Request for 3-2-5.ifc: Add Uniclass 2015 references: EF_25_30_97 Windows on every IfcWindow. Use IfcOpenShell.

First a look at what the model holds.

```python
import ifcopenshell

model = ifcopenshell.open("3-2-5.ifc")
print(model.schema)
print("classifications:", [c.Name for c in model.by_type("IfcClassification")])
for ifc_class in ("IfcDoor", "IfcRoof", "IfcStair", "IfcWall", "IfcWindow"):
    print(ifc_class, len(model.by_type(ifc_class)))
```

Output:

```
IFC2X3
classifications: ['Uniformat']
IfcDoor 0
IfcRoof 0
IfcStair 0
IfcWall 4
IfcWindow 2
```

```python
import ifcopenshell
import ifcopenshell.api.classification

model = ifcopenshell.open("3-2-5.ifc")

# IFC2X3 requires Source and Edition and has no link from the project to the system.
system = model.create_entity("IfcClassification", Source="NBS", Edition="2015", Name="Uniclass 2015")

codes = {
    "IfcWindow": ("EF_25_30_97", "Windows"),
}
for ifc_class, (code, name) in codes.items():
    products = model.by_type(ifc_class)
    ifcopenshell.api.classification.add_reference(
        model, products=products, classification=system, identification=code, name=name
    )
    print(code, len(products))

model.write("3-2-5-out.ifc")
```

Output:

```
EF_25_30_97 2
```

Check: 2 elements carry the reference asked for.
